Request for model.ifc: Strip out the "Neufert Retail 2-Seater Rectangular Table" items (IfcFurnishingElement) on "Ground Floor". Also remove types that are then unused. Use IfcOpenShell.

First a look at what the model holds.

```python
import ifcopenshell
import ifcopenshell.util.element

model = ifcopenshell.open("model.ifc")
print(model.schema)
storey = next(s for s in model.by_type("IfcBuildingStorey") if s.Name == "Ground Floor")
furniture = [e for e in ifcopenshell.util.element.get_decomposition(storey) if e.is_a("IfcFurnishingElement")]
seen = {}
for e in furniture:
    element_type = ifcopenshell.util.element.get_type(e)
    name = element_type.Name if element_type not in (None, e) else None
    seen[name] = seen.get(name, 0) + 1
for name, count in sorted(seen.items(), key=str):
    print(count, "x", name)
```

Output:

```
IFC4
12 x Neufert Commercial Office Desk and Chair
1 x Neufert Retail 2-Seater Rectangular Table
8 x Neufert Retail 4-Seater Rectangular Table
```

```python
import ifcopenshell
import ifcopenshell.api.root
import ifcopenshell.util.element

model = ifcopenshell.open("model.ifc")

storey = next(s for s in model.by_type("IfcBuildingStorey") if s.Name == "Ground Floor")
furniture = [e for e in ifcopenshell.util.element.get_decomposition(storey) if e.is_a("IfcFurnishingElement")]
targets = [e for e in furniture if (t := ifcopenshell.util.element.get_type(e)) not in (None, e) and t.Name == "Neufert Retail 2-Seater Rectangular Table"]
types = {ifcopenshell.util.element.get_type(e) for e in targets} - {None, *targets}

for e in targets:
    ifcopenshell.api.root.remove_product(model, product=e)
print(len(targets), "removed")

unused = [t for t in types if not ifcopenshell.util.element.get_types(t)]
for t in unused:
    ifcopenshell.api.root.remove_product(model, product=t)
print(len(unused), "unused types removed")

model.write("model-out.ifc")
```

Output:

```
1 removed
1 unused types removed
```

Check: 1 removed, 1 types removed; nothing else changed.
